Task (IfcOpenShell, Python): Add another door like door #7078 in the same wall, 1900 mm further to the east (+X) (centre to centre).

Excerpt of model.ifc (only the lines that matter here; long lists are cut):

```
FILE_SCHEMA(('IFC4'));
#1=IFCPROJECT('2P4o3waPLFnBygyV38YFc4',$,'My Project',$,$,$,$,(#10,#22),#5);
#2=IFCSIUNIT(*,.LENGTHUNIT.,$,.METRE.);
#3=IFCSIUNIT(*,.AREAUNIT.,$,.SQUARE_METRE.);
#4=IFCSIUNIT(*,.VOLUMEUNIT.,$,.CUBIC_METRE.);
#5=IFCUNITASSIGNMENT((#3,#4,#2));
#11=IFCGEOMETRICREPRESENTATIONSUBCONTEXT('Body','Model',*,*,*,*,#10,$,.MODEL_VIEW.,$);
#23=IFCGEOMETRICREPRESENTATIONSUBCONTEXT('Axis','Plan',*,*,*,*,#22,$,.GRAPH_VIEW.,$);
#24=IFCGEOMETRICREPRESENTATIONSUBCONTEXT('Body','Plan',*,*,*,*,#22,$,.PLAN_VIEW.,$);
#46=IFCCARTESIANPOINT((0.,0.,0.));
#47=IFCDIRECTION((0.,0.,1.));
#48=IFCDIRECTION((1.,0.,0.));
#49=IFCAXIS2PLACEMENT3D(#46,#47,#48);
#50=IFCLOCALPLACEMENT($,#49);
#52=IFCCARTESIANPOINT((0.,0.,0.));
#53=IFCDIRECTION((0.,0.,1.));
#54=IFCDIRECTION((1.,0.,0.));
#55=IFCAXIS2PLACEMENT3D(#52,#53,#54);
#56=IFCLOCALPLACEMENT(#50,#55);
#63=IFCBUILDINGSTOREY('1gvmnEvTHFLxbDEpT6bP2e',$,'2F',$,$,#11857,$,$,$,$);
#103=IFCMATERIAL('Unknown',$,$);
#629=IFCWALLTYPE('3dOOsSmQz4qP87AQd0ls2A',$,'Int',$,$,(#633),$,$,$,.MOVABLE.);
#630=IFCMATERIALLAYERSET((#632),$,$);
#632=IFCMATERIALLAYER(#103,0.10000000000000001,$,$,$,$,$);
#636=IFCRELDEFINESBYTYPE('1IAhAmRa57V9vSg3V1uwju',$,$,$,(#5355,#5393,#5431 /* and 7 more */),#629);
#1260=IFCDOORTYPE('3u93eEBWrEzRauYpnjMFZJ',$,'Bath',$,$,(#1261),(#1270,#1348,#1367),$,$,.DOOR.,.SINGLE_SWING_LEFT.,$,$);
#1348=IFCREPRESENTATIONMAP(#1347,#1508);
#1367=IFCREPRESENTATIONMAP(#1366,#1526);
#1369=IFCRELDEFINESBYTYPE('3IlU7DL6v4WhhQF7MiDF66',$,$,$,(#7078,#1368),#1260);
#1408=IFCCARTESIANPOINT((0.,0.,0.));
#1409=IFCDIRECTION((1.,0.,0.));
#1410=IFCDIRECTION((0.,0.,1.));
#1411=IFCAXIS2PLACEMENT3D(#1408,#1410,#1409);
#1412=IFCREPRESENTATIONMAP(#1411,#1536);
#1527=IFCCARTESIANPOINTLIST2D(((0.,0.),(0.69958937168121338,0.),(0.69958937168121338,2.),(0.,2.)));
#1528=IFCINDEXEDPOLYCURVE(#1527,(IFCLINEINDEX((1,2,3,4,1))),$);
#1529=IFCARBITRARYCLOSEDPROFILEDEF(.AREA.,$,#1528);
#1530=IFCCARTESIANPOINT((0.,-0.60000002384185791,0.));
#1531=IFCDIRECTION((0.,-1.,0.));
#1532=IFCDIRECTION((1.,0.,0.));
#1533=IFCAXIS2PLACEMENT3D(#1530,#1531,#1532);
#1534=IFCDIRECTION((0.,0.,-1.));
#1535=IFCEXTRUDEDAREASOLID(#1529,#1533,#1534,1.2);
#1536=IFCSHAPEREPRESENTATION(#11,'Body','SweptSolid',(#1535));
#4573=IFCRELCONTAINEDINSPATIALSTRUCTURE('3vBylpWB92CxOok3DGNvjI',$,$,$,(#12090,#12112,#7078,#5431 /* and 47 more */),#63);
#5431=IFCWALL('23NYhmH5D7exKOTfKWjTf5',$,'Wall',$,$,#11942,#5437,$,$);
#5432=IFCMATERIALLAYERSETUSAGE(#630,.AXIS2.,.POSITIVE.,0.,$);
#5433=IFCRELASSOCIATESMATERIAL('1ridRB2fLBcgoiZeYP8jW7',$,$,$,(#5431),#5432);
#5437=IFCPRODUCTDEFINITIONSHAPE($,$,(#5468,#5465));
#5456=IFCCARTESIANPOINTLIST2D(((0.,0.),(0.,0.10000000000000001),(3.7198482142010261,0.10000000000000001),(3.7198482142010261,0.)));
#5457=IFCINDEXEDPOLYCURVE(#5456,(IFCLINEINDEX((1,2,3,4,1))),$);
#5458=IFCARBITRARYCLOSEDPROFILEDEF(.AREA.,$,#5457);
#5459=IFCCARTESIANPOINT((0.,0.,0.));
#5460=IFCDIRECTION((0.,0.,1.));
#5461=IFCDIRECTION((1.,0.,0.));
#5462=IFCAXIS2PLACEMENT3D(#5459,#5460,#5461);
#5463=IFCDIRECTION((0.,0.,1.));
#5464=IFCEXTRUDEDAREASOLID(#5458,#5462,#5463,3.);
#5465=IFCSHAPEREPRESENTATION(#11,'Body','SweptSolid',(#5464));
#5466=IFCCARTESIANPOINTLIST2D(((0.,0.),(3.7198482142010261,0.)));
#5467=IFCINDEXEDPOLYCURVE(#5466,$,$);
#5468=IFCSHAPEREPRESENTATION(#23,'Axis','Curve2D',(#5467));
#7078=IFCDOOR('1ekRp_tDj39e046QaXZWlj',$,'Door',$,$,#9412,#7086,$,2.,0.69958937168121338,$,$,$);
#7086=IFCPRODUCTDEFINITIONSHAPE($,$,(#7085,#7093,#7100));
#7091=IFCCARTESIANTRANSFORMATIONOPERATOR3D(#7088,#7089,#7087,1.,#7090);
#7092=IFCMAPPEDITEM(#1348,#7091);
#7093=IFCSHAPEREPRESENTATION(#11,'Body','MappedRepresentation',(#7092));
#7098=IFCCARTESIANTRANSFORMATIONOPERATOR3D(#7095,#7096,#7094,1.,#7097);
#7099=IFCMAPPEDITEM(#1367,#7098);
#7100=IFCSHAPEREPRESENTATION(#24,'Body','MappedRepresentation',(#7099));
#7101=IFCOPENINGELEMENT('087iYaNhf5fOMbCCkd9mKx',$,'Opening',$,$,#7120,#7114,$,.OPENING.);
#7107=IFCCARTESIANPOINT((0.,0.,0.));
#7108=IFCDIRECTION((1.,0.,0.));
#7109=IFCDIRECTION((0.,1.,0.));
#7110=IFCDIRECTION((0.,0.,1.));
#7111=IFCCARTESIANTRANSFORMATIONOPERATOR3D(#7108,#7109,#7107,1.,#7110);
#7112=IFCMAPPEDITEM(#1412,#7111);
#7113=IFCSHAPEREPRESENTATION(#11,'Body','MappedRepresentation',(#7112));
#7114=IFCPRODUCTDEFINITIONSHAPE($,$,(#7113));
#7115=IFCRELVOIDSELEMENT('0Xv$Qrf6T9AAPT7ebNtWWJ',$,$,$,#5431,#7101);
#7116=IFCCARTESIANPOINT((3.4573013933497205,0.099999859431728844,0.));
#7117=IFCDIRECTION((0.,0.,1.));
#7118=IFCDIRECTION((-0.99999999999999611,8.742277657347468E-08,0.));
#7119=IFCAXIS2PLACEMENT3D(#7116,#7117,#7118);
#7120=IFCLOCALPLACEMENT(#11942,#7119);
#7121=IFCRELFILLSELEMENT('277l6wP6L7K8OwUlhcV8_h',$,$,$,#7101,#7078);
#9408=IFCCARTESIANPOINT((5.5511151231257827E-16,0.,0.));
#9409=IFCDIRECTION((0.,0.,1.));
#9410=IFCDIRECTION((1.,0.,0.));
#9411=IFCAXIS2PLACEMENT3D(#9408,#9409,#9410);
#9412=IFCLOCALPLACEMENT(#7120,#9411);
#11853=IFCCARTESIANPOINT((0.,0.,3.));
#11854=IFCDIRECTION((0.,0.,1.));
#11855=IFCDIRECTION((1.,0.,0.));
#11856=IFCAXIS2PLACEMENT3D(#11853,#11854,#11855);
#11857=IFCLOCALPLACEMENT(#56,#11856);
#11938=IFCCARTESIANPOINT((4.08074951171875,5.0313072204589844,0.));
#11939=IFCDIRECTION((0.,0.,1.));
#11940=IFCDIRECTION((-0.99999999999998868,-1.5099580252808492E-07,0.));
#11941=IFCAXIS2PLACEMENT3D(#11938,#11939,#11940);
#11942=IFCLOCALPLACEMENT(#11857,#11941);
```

```python
import ifcopenshell
import ifcopenshell.api.feature
import ifcopenshell.api.geometry
import ifcopenshell.api.root
import ifcopenshell.geom
import ifcopenshell.util.element
import ifcopenshell.util.placement
import ifcopenshell.util.shape
import ifcopenshell.util.unit

model = ifcopenshell.open("model.ifc")
unit_scale = ifcopenshell.util.unit.calculate_unit_scale(model)
settings = ifcopenshell.geom.settings()


def volume(element):
    """Net volume in cubic metres, openings subtracted."""
    shape = ifcopenshell.geom.create_shape(settings, element)
    return ifcopenshell.util.shape.get_volume(shape.geometry)


door = model.by_guid("1ekRp_tDj39e046QaXZWlj")
opening = door.FillsVoids[0].RelatingOpeningElement
wall = opening.VoidsElements[0].RelatingBuildingElement
before = volume(wall)
shift = ifcopenshell.util.placement.get_local_placement(wall.ObjectPlacement)[:3, 0] * -1.9 / unit_scale

# copy_class copies the void relationship, type, container and properties, but no geometry.
new_opening = ifcopenshell.api.root.copy_class(model, product=opening)
new_opening.Representation = ifcopenshell.util.element.copy_deep(
    model, opening.Representation, exclude=["IfcGeometricRepresentationContext", "IfcRepresentationMap"]
)
new_door = ifcopenshell.api.root.copy_class(model, product=door)
new_door.Representation = ifcopenshell.util.element.copy_deep(
    model, door.Representation, exclude=["IfcGeometricRepresentationContext", "IfcRepresentationMap"]
)
ifcopenshell.api.feature.add_filling(model, opening=new_opening, element=new_door)

for old, new in ((opening, new_opening), (door, new_door)):
    matrix = ifcopenshell.util.placement.get_local_placement(old.ObjectPlacement)
    matrix[:3, 3] += shift
    ifcopenshell.api.geometry.edit_object_placement(model, product=new, matrix=matrix, is_si=False)

after = volume(wall)

print(f"wall volume {before:.3f} -> {after:.3f} m3")

model.write("model_edited.ifc")
```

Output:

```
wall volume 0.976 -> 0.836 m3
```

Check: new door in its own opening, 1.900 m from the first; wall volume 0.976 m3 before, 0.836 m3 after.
